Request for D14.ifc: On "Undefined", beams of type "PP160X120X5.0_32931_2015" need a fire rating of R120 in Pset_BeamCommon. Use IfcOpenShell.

First a look at what the model holds.

```python
import ifcopenshell
import ifcopenshell.util.element

model = ifcopenshell.open("D14.ifc")
print(model.schema)
storey = next(s for s in model.by_type("IfcBuildingStorey") if s.Name == "Undefined")
beams = [e for e in ifcopenshell.util.element.get_decomposition(storey) if e.is_a("IfcBeam")]
seen = {}
for e in beams:
    element_type = ifcopenshell.util.element.get_type(e)
    key = (element_type.Name if element_type != e and element_type else None, ifcopenshell.util.element.get_pset(e, "Pset_BeamCommon", "FireRating"))
    seen[key] = seen.get(key, 0) + 1
for (name, value), count in sorted(seen.items(), key=str):
    print(count, "x", name, "|", value)
```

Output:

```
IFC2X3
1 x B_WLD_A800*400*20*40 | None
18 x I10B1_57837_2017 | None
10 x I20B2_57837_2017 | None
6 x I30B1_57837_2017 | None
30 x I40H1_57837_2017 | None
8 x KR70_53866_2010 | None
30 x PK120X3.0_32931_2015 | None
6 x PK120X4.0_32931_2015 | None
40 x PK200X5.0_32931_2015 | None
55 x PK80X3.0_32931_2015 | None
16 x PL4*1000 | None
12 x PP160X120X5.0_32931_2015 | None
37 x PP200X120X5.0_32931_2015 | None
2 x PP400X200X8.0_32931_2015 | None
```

```python
import ifcopenshell
import ifcopenshell.api.pset
import ifcopenshell.util.element

model = ifcopenshell.open("D14.ifc")

storey = next(s for s in model.by_type("IfcBuildingStorey") if s.Name == "Undefined")
beams = [e for e in ifcopenshell.util.element.get_decomposition(storey) if e.is_a("IfcBeam")]

count = 0
for e in beams:
    element_type = ifcopenshell.util.element.get_type(e)
    if element_type in (None, e) or element_type.Name != "PP160X120X5.0_32931_2015":
        continue
    found = ifcopenshell.util.element.get_pset(e, "Pset_BeamCommon", should_inherit=False)
    if found:
        pset = model.by_id(found["id"])
        if len(ifcopenshell.util.element.get_elements_by_pset(pset)) > 1:
            pset = ifcopenshell.api.pset.unshare_pset(model, products=[e], pset=pset)[0]
    else:
        pset = ifcopenshell.api.pset.add_pset(model, product=e, name="Pset_BeamCommon")
    ifcopenshell.api.pset.edit_pset(model, pset=pset, properties={"FireRating": "R120"})
    count += 1

print(count, "beams updated")

model.write("D14_v2.ifc")
```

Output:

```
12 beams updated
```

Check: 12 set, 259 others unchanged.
